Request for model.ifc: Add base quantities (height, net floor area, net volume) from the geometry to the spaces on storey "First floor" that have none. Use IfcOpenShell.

First a look at what the model holds.

```python
import ifcopenshell
import ifcopenshell.util.element
import ifcopenshell.util.unit

model = ifcopenshell.open("model.ifc")
print(model.schema)
for unit_type in ("LENGTHUNIT", "AREAUNIT", "VOLUMEUNIT"):
    print(unit_type, ifcopenshell.util.unit.calculate_unit_scale(model, unit_type))
storey = next(s for s in model.by_type("IfcBuildingStorey") if s.Name == "First floor")
spaces = [e for e in ifcopenshell.util.element.get_decomposition(storey) if e.is_a("IfcSpace")]
for e in sorted(spaces, key=lambda e: e.id()):
    print(e.id(), e.is_a(), e.Name, list(ifcopenshell.util.element.get_psets(e, qtos_only=True)), sep=" | ")
```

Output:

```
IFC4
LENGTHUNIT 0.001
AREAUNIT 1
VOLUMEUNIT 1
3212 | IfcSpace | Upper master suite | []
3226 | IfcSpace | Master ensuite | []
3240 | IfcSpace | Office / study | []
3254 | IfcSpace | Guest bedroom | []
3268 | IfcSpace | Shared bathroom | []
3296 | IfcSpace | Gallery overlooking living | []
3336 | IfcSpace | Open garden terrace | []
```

```python
import ifcopenshell
import ifcopenshell.api.pset
import ifcopenshell.geom
import ifcopenshell.util.element
import ifcopenshell.util.shape
import ifcopenshell.util.unit

model = ifcopenshell.open("model.ifc")
unit_scale = ifcopenshell.util.unit.calculate_unit_scale(model)
area_scale = ifcopenshell.util.unit.calculate_unit_scale(model, "AREAUNIT")
volume_scale = ifcopenshell.util.unit.calculate_unit_scale(model, "VOLUMEUNIT")
settings = ifcopenshell.geom.settings()

storey = next(s for s in model.by_type("IfcBuildingStorey") if s.Name == "First floor")
spaces = [e for e in ifcopenshell.util.element.get_decomposition(storey) if e.is_a("IfcSpace")]

for e in sorted(spaces, key=lambda e: e.id()):
    if ifcopenshell.util.element.get_psets(e, qtos_only=True, should_inherit=False):
        continue
    # Geometry comes back in metres, in the element's own axes.
    shape = ifcopenshell.geom.create_shape(settings, e)
    values = {
        "Height": ifcopenshell.util.shape.get_z(shape.geometry) / unit_scale,
        "NetFloorArea": ifcopenshell.util.shape.get_footprint_area(shape.geometry) / area_scale,
        "NetVolume": ifcopenshell.util.shape.get_volume(shape.geometry) / volume_scale,
    }
    qto = ifcopenshell.api.pset.add_qto(model, product=e, name="Qto_SpaceBaseQuantities")
    ifcopenshell.api.pset.edit_qto(model, qto=qto, properties=values)
    print(e.id(), {k: round(v, 3) for k, v in values.items()})

model.write("model_edited.ifc")
```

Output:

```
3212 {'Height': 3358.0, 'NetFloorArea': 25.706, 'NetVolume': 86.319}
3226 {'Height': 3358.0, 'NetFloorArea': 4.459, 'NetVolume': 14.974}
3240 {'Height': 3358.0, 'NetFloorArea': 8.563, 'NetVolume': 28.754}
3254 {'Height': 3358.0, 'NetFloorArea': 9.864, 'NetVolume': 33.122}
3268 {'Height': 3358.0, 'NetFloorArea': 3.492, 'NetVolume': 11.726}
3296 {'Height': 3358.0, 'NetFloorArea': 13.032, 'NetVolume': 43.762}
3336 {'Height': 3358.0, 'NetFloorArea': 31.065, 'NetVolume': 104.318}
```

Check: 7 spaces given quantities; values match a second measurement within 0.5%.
